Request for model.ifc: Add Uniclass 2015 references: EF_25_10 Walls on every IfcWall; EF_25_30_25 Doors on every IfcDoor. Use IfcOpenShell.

First a look at what the model holds.

```python
import ifcopenshell

model = ifcopenshell.open("model.ifc")
print(model.schema)
print("classifications:", [c.Name for c in model.by_type("IfcClassification")])
for ifc_class in ("IfcDoor", "IfcRoof", "IfcStair", "IfcWall", "IfcWindow"):
    print(ifc_class, len(model.by_type(ifc_class)))
```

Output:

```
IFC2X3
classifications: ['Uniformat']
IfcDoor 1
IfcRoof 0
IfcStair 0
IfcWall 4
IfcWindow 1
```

```python
import ifcopenshell
import ifcopenshell.api.classification

model = ifcopenshell.open("model.ifc")

# IFC2X3 requires Source and Edition and has no link from the project to the system.
system = model.create_entity("IfcClassification", Source="NBS", Edition="2015", Name="Uniclass 2015")

codes = {
    "IfcWall": ("EF_25_10", "Walls"),
    "IfcDoor": ("EF_25_30_25", "Doors"),
}
for ifc_class, (code, name) in codes.items():
    products = model.by_type(ifc_class)
    ifcopenshell.api.classification.add_reference(
        model, products=products, classification=system, identification=code, name=name
    )
    print(code, len(products))

model.write("model_rev.ifc")
```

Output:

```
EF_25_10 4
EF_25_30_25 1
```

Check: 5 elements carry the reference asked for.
